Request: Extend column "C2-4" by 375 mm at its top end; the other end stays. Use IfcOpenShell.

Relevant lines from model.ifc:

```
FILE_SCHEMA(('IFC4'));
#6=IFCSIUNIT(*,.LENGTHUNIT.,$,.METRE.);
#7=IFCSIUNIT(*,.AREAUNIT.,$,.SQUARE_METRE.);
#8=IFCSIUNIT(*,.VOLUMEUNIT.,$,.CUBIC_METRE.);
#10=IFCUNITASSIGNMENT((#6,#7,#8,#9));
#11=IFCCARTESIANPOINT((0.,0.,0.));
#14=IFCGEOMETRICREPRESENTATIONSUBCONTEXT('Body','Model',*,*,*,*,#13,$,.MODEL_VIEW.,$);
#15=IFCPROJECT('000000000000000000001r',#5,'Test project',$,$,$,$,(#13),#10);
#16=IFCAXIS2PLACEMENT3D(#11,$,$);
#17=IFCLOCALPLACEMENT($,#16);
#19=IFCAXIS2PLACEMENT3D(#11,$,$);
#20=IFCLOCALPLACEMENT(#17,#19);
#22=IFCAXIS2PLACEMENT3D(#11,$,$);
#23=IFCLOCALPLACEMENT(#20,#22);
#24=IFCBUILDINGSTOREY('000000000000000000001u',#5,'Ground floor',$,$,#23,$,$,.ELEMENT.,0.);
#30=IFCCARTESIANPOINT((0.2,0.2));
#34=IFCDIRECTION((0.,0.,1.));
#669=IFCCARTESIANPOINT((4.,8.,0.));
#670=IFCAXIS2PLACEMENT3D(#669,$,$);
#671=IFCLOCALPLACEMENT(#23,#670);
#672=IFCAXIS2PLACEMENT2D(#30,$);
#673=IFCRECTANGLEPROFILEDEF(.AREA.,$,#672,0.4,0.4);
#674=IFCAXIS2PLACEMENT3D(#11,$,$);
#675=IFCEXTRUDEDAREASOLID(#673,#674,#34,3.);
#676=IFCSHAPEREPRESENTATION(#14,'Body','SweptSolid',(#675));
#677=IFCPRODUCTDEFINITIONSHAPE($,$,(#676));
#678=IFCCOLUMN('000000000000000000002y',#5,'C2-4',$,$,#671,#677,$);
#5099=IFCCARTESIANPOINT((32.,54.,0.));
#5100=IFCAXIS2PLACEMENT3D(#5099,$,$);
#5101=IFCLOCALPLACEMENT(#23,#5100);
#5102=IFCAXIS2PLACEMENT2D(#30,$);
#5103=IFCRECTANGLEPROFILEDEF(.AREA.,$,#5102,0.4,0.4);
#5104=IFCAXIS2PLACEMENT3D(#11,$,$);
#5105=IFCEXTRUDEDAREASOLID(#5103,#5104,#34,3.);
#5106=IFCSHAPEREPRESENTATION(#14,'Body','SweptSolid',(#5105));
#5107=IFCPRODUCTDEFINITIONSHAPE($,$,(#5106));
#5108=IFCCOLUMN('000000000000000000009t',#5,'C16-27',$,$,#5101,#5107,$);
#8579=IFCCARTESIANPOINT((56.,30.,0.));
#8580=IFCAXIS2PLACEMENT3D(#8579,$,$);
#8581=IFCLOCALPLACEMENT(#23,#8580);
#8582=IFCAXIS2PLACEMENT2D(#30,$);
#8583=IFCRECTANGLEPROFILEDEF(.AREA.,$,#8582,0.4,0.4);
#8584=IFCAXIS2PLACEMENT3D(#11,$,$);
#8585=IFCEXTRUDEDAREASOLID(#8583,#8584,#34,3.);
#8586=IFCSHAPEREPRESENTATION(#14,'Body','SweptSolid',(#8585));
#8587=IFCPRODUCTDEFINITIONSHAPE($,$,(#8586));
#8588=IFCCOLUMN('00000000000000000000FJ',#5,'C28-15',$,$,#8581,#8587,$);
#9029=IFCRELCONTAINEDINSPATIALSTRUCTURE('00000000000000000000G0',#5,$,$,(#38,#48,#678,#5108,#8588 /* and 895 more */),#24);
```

```python
import ifcopenshell
import ifcopenshell.util.representation
import ifcopenshell.util.unit

model = ifcopenshell.open("model.ifc")
unit_scale = ifcopenshell.util.unit.calculate_unit_scale(model)

member = model.by_guid("000000000000000000002y")
change = 0.375 / unit_scale

# The extrusion runs towards the end named, so only its depth changes.
body = ifcopenshell.util.representation.get_representation(member, "Model", "Body")
solid = body.Items[0]
old_length = solid.Depth
solid.Depth += change

print(f"length {old_length:g} -> {solid.Depth:g}")

model.write("model_updated.ifc")
```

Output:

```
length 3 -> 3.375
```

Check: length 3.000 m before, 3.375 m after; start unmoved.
